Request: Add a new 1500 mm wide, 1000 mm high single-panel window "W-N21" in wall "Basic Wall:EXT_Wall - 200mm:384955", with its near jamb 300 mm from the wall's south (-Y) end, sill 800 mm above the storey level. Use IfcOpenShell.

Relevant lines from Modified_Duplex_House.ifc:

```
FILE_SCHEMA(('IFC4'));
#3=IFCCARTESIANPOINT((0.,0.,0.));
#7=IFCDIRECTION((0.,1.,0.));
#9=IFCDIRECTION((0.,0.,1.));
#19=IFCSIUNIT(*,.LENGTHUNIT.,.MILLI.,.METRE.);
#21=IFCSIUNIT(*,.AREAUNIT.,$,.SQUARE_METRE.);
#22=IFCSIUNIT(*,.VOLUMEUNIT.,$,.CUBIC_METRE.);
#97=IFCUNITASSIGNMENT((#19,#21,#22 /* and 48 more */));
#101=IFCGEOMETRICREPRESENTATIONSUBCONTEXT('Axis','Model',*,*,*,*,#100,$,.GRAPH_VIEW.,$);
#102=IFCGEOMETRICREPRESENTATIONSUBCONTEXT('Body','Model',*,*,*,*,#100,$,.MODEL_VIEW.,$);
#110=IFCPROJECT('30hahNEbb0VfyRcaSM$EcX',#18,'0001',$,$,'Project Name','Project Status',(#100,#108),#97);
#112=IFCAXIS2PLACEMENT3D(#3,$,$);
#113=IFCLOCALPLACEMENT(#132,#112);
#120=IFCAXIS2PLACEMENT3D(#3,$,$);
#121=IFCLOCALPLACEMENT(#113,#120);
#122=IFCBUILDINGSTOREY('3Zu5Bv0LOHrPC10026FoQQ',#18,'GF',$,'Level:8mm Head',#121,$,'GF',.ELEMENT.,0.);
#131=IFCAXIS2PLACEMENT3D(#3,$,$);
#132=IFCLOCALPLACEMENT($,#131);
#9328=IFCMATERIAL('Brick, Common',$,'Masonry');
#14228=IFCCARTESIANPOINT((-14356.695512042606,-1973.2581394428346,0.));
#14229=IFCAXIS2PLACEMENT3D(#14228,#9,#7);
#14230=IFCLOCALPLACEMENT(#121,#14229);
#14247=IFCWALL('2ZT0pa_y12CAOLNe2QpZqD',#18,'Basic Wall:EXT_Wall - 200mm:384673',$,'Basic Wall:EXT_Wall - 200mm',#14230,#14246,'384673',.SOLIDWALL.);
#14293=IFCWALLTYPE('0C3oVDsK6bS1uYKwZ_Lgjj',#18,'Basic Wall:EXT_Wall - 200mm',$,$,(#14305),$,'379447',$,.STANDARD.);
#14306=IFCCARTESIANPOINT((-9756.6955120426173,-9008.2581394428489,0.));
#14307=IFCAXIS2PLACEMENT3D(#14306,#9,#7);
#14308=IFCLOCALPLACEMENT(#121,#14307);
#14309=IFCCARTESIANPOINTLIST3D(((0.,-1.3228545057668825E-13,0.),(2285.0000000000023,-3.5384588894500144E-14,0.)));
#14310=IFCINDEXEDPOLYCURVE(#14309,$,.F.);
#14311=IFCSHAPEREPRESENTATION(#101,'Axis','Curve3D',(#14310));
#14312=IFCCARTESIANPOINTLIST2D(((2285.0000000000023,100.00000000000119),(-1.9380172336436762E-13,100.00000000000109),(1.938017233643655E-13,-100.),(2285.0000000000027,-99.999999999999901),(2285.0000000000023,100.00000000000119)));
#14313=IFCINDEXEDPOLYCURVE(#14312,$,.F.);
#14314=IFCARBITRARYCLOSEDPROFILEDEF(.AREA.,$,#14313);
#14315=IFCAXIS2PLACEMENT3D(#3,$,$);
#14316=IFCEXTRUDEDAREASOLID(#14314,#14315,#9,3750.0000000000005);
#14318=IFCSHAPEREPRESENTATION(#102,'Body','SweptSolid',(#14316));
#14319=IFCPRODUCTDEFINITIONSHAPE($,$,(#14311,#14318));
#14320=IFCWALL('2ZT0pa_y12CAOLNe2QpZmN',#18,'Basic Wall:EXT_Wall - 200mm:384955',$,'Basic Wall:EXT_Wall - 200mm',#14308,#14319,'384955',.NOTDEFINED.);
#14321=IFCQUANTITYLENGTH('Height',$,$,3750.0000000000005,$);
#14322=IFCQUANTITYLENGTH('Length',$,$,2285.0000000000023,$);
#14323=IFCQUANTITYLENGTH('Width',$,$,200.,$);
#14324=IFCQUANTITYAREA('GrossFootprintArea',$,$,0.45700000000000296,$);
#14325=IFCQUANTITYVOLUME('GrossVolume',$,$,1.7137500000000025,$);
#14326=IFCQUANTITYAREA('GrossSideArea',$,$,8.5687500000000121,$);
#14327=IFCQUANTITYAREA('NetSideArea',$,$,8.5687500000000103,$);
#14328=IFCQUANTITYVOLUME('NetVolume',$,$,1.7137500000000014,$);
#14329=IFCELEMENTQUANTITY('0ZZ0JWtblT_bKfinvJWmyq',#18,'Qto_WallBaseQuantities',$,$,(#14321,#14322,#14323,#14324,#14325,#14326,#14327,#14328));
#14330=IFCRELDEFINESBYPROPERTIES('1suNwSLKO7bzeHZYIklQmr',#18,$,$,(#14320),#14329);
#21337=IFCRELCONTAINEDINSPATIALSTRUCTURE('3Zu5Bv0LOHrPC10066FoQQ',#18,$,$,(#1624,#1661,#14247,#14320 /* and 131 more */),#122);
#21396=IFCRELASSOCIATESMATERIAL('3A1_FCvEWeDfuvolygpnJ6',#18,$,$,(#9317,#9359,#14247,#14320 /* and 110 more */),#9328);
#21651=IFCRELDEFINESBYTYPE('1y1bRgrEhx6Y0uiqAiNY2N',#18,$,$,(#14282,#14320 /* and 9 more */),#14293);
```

```python
import numpy as np
import ifcopenshell
import ifcopenshell.api.feature
import ifcopenshell.api.geometry
import ifcopenshell.api.pset
import ifcopenshell.api.root
import ifcopenshell.api.spatial
import ifcopenshell.geom
import ifcopenshell.util.element
import ifcopenshell.util.placement
import ifcopenshell.util.representation
import ifcopenshell.util.shape
import ifcopenshell.util.unit

model = ifcopenshell.open("Modified_Duplex_House.ifc")
unit_scale = ifcopenshell.util.unit.calculate_unit_scale(model)
area_scale = ifcopenshell.util.unit.calculate_unit_scale(model, "AREAUNIT")
volume_scale = ifcopenshell.util.unit.calculate_unit_scale(model, "VOLUMEUNIT")
settings = ifcopenshell.geom.settings()


def volume(element):
    """Net volume in cubic metres, openings subtracted."""
    shape = ifcopenshell.geom.create_shape(settings, element)
    return ifcopenshell.util.shape.get_volume(shape.geometry)


wall = model.by_guid("2ZT0pa_y12CAOLNe2QpZmN")
storey = ifcopenshell.util.element.get_container(wall, ifc_class="IfcBuildingStorey")
context = ifcopenshell.util.representation.get_context(model, "Model", "Body", "MODEL_VIEW")
before = volume(wall)

width, height, from_end, sill = 1.5, 1, 0.3, 0.8  # metres

# The wall runs along its own X axis, and the end named is its -X end.
wall_shape = ifcopenshell.geom.create_shape(settings, wall)
x, y, z = ifcopenshell.util.shape.get_vertices(wall_shape.geometry).T
start = x.min() + from_end
face, thickness = float(y.min()), float(y.max() - y.min())
wall_matrix = ifcopenshell.util.placement.get_local_placement(wall.ObjectPlacement)
level = ifcopenshell.util.placement.get_local_placement(storey.ObjectPlacement)[2, 3]


def in_wall(x, y):
    """Placement at x, y metres in the wall's axes, at sill height."""
    matrix = wall_matrix.copy()
    matrix[:, 3] = wall_matrix @ np.array([x / unit_scale, y / unit_scale, 0.0, 1.0])
    matrix[2, 3] = level + sill / unit_scale
    return matrix


# Opening: a box that overshoots both wall faces by 50 mm.
opening = ifcopenshell.api.root.create_entity(model, ifc_class="IfcOpeningElement", predefined_type="OPENING")
box = ifcopenshell.api.geometry.add_wall_representation(
    model, context=context, length=width, height=height, thickness=thickness + 0.1
)
ifcopenshell.api.geometry.assign_representation(model, product=opening, representation=box)
ifcopenshell.api.geometry.edit_object_placement(model, product=opening, matrix=in_wall(start, face - 0.05), is_si=False)
ifcopenshell.api.feature.add_feature(model, feature=opening, element=wall)

window = ifcopenshell.api.root.create_entity(model, ifc_class="IfcWindow", name="W-N21", predefined_type="WINDOW")
window.OverallWidth, window.OverallHeight = width / unit_scale, height / unit_scale
window.PartitioningType = "SINGLE_PANEL"
body = ifcopenshell.api.geometry.add_window_representation(
    model,
    context=context,
    overall_width=window.OverallWidth,
    overall_height=window.OverallHeight,
    partition_type="SINGLE_PANEL",
)
ifcopenshell.api.geometry.assign_representation(model, product=window, representation=body)
ifcopenshell.api.spatial.assign_container(model, products=[window], relating_structure=storey)
ifcopenshell.api.feature.add_filling(model, opening=opening, element=window)

# Centre the window in the wall's thickness.
ifcopenshell.api.geometry.edit_object_placement(model, product=window, matrix=in_wall(start, face), is_si=False)
window_shape = ifcopenshell.geom.create_shape(settings, window)
depth = ifcopenshell.util.shape.get_vertices(window_shape.geometry)[:, 1]
offset = face + thickness / 2 - (depth.min() + depth.max()) / 2
ifcopenshell.api.geometry.edit_object_placement(model, product=window, matrix=in_wall(start, offset), is_si=False)

after = volume(wall)

# Update the wall's stored quantities.
qto = model.by_id(ifcopenshell.util.element.get_pset(wall, "Qto_WallBaseQuantities", should_inherit=False)["id"])
ifcopenshell.api.pset.edit_qto(model, qto=qto, properties={
    "NetSideArea": after / thickness / area_scale,
    "NetVolume": after / volume_scale,
})

print(f"wall volume {before:.3f} -> {after:.3f} m3")

model.write("Modified_Duplex_House_v2.ifc")
```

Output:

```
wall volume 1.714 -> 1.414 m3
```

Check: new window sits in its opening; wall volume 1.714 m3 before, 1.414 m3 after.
